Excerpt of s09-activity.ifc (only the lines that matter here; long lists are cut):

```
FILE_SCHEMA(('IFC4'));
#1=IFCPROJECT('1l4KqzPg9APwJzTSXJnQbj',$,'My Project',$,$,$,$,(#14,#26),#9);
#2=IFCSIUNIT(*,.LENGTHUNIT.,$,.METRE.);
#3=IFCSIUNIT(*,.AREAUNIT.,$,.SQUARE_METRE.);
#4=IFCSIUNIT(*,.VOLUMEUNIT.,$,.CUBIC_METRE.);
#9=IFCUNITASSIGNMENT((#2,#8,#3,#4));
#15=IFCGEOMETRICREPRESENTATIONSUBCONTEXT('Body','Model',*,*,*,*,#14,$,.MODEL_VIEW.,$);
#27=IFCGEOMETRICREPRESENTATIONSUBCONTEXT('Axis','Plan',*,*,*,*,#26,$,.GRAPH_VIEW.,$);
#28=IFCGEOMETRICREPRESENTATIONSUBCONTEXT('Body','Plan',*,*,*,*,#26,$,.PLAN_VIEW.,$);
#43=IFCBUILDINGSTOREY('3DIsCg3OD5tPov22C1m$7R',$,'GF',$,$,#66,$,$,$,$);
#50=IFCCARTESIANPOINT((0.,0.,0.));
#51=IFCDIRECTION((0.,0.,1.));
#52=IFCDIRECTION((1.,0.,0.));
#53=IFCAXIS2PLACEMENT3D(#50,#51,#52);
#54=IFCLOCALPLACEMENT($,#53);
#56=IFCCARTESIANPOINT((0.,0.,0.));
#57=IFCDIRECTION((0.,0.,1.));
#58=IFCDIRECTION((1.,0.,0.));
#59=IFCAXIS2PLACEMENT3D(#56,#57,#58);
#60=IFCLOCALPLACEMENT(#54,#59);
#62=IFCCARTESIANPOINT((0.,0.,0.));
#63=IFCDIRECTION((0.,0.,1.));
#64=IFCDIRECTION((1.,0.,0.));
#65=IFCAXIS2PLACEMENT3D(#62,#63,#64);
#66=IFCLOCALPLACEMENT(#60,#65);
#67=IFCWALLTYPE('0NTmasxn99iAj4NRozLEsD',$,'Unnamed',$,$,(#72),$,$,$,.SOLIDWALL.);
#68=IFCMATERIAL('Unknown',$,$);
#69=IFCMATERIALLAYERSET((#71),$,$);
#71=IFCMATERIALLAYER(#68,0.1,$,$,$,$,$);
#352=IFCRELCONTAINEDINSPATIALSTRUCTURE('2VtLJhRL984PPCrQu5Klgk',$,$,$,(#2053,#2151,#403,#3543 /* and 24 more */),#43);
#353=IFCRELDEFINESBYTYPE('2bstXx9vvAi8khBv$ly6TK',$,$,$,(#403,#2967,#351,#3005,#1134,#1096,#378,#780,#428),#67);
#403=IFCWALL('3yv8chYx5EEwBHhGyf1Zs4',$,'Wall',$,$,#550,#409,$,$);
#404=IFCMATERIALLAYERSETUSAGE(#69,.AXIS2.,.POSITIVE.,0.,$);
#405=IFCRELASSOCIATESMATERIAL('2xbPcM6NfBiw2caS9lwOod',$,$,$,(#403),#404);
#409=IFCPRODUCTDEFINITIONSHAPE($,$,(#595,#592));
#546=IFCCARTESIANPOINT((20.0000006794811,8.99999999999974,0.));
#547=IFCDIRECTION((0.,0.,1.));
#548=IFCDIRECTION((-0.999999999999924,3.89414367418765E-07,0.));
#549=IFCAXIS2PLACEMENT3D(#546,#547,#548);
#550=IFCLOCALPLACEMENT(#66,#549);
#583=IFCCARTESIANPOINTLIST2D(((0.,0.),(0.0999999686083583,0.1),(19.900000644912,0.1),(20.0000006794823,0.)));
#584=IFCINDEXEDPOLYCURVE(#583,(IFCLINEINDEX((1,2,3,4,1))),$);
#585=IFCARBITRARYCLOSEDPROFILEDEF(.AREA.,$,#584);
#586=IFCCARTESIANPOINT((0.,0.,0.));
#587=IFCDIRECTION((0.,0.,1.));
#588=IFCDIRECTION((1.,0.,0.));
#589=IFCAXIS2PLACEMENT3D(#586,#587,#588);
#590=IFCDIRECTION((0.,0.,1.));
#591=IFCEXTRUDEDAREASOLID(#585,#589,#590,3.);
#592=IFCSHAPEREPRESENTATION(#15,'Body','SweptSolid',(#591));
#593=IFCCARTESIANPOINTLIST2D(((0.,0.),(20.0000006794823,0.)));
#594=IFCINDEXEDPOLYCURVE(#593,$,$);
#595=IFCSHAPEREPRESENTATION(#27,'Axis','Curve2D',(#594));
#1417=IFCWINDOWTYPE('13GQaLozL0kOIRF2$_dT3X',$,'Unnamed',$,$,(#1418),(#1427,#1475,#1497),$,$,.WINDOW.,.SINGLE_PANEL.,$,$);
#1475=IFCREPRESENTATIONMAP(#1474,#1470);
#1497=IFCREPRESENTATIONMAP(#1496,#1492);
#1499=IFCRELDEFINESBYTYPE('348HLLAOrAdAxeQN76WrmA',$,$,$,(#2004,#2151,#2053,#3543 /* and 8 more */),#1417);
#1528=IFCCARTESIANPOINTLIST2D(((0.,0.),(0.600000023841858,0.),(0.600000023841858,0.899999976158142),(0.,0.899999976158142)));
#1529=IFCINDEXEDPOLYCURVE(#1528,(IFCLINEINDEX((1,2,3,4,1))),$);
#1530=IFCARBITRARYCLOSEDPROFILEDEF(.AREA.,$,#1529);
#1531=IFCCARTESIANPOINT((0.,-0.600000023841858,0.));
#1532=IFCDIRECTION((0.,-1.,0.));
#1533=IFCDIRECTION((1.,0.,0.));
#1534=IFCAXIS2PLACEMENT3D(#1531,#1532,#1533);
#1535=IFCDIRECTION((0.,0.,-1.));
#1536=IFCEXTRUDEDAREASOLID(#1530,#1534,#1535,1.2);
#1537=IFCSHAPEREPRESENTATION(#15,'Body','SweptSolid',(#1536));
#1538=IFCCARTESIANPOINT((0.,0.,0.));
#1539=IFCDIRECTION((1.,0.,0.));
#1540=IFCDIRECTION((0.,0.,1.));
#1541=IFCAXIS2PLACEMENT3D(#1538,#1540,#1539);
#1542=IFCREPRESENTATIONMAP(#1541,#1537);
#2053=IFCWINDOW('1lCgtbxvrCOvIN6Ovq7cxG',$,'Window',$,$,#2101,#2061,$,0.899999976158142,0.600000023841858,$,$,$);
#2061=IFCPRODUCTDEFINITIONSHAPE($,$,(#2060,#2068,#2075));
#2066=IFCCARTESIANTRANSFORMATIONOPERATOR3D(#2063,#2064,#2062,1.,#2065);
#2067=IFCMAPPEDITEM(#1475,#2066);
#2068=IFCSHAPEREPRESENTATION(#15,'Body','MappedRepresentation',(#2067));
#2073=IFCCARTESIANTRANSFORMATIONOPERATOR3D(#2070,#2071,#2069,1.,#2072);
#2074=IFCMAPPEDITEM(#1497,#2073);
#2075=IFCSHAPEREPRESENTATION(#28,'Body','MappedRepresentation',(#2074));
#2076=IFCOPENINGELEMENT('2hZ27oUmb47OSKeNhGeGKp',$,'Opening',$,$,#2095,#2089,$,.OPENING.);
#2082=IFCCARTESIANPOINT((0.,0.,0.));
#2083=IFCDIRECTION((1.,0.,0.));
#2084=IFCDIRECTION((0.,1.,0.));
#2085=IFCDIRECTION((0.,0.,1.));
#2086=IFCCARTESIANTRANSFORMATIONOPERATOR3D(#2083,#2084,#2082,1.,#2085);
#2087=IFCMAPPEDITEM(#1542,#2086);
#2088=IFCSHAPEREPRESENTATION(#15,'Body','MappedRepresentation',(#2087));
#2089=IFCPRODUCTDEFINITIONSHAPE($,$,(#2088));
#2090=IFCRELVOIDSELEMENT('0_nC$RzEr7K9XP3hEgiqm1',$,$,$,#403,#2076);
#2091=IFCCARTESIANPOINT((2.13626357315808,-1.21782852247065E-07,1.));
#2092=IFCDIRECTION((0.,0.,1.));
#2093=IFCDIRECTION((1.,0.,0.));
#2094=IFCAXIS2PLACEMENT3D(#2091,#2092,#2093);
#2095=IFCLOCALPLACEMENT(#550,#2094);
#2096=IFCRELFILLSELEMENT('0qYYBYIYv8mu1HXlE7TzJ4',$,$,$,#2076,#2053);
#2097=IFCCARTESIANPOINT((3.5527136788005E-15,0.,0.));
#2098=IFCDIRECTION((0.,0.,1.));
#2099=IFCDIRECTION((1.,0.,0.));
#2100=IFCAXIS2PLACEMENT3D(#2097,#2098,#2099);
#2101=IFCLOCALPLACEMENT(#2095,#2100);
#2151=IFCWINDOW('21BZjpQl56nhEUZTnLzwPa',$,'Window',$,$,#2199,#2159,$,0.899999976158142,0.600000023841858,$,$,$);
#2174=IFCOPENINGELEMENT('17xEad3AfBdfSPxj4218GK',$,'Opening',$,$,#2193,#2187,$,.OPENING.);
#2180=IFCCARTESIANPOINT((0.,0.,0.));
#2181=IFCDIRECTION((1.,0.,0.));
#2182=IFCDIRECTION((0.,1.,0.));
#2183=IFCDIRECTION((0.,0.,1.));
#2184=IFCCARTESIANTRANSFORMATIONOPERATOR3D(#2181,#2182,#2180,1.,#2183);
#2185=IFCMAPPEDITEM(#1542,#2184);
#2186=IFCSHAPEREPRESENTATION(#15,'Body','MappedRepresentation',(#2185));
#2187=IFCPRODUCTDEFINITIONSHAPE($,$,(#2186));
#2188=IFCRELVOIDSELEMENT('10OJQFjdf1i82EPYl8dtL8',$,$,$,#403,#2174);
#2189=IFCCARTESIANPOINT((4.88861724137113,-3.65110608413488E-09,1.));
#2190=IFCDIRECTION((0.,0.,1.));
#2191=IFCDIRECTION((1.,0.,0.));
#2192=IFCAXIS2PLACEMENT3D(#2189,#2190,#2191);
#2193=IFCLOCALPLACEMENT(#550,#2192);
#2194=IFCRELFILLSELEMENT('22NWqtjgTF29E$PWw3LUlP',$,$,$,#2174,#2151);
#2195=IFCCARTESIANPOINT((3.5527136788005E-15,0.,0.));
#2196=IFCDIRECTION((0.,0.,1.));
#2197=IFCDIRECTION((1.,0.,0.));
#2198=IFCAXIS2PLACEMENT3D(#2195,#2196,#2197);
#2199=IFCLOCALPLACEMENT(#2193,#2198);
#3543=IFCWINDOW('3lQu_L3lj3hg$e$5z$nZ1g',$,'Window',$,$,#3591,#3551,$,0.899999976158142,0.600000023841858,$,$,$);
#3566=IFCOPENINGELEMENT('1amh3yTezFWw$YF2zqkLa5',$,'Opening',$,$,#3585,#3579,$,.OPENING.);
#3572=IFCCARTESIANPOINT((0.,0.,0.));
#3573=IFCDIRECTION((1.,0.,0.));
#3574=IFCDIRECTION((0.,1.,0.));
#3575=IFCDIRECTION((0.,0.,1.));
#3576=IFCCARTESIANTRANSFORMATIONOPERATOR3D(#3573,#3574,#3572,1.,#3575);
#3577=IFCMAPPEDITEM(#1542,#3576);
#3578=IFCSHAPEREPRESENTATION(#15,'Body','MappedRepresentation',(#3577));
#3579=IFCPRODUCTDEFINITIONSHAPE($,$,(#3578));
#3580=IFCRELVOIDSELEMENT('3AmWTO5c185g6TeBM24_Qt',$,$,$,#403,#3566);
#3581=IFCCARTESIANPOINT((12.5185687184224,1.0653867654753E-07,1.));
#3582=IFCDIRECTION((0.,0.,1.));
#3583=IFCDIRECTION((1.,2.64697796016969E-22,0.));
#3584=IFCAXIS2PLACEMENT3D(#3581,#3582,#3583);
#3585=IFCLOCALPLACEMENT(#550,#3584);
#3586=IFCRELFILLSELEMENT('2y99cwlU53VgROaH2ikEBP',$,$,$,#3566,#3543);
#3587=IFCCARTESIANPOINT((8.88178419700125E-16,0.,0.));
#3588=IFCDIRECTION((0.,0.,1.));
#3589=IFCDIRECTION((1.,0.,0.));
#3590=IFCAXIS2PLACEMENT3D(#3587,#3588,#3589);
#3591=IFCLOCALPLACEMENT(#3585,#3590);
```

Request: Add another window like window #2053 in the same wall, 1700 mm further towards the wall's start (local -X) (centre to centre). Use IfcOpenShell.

```python
import ifcopenshell
import ifcopenshell.api.feature
import ifcopenshell.api.geometry
import ifcopenshell.api.root
import ifcopenshell.geom
import ifcopenshell.util.element
import ifcopenshell.util.placement
import ifcopenshell.util.shape
import ifcopenshell.util.unit

model = ifcopenshell.open("s09-activity.ifc")
unit_scale = ifcopenshell.util.unit.calculate_unit_scale(model)
settings = ifcopenshell.geom.settings()


def volume(element):
    """Net volume in cubic metres, openings subtracted."""
    shape = ifcopenshell.geom.create_shape(settings, element)
    return ifcopenshell.util.shape.get_volume(shape.geometry)


window = model.by_guid("1lCgtbxvrCOvIN6Ovq7cxG")
opening = window.FillsVoids[0].RelatingOpeningElement
wall = opening.VoidsElements[0].RelatingBuildingElement
before = volume(wall)
shift = ifcopenshell.util.placement.get_local_placement(wall.ObjectPlacement)[:3, 0] * -1.7 / unit_scale

# copy_class copies the void relationship, type, container and properties, but no geometry.
new_opening = ifcopenshell.api.root.copy_class(model, product=opening)
new_opening.Representation = ifcopenshell.util.element.copy_deep(
    model, opening.Representation, exclude=["IfcGeometricRepresentationContext", "IfcRepresentationMap"]
)
new_window = ifcopenshell.api.root.copy_class(model, product=window)
new_window.Representation = ifcopenshell.util.element.copy_deep(
    model, window.Representation, exclude=["IfcGeometricRepresentationContext", "IfcRepresentationMap"]
)
ifcopenshell.api.feature.add_filling(model, opening=new_opening, element=new_window)

for old, new in ((opening, new_opening), (window, new_window)):
    matrix = ifcopenshell.util.placement.get_local_placement(old.ObjectPlacement)
    matrix[:3, 3] += shift
    ifcopenshell.api.geometry.edit_object_placement(model, product=new, matrix=matrix, is_si=False)

after = volume(wall)

print(f"wall volume {before:.3f} -> {after:.3f} m3")

model.write("s09-activity_rev.ifc")
```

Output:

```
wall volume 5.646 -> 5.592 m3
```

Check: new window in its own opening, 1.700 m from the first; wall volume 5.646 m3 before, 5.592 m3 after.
